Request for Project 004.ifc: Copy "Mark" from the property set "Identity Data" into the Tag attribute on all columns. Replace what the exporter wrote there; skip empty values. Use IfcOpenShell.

First a look at what the model holds.

```python
import ifcopenshell
import ifcopenshell.util.element

model = ifcopenshell.open("Project 004.ifc")
print(model.schema)
columns = model.by_type("IfcColumn")
print(len(columns), "columns")
for e in columns[:8]:
    source = ifcopenshell.util.element.get_pset(e, "Identity Data", "Mark")
    target = e.Tag
    print(e.id(), repr(source), repr(target), sep=" | ")
```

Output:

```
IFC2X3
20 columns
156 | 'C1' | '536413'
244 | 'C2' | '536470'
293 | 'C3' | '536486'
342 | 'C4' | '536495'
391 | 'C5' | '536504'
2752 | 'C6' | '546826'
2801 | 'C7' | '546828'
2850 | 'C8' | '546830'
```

```python
import ifcopenshell
import ifcopenshell.util.element

model = ifcopenshell.open("Project 004.ifc")

count = 0
for e in model.by_type("IfcColumn"):
    value = ifcopenshell.util.element.get_pset(e, "Identity Data", "Mark")
    current = e.Tag
    if not value or not value.strip() or current == value:
        continue
    e.Tag = value
    count += 1

print(count, "columns updated")

model.write("Project 004-out.ifc")
```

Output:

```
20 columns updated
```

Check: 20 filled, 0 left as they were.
